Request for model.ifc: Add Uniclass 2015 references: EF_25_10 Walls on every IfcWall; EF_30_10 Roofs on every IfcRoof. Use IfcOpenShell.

First a look at what the model holds.

```python
import ifcopenshell

model = ifcopenshell.open("model.ifc")
print(model.schema)
print("classifications:", [c.Name for c in model.by_type("IfcClassification")])
for ifc_class in ("IfcDoor", "IfcRoof", "IfcStair", "IfcWall", "IfcWindow"):
    print(ifc_class, len(model.by_type(ifc_class)))
```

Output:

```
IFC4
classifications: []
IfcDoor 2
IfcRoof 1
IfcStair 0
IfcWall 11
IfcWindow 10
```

```python
import ifcopenshell
import ifcopenshell.api.classification

model = ifcopenshell.open("model.ifc")

system = ifcopenshell.api.classification.add_classification(model, classification="Uniclass 2015")

codes = {
    "IfcWall": ("EF_25_10", "Walls"),
    "IfcRoof": ("EF_30_10", "Roofs"),
}
for ifc_class, (code, name) in codes.items():
    products = model.by_type(ifc_class)
    ifcopenshell.api.classification.add_reference(
        model, products=products, classification=system, identification=code, name=name
    )
    print(code, len(products))

model.write("model_rev.ifc")
```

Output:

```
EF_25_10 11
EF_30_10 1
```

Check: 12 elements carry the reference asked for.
